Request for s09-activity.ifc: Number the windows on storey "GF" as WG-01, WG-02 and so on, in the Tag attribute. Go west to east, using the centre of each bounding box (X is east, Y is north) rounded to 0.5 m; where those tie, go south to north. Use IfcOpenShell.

First a look at what the model holds.

```python
import ifcopenshell
import ifcopenshell.util.element
import ifcopenshell.util.placement

model = ifcopenshell.open("s09-activity.ifc")
print(model.schema)
storey = next(s for s in model.by_type("IfcBuildingStorey") if s.Name == "GF")
windows = [e for e in ifcopenshell.util.element.get_decomposition(storey) if e.is_a("IfcWindow")]
for e in sorted(windows, key=lambda e: e.id()):
    origin = ifcopenshell.util.placement.get_local_placement(e.ObjectPlacement)[:3, 3]
    print(e.id(), e.Tag, e.Name, origin.round(2) + 0.0, sep=" | ")
```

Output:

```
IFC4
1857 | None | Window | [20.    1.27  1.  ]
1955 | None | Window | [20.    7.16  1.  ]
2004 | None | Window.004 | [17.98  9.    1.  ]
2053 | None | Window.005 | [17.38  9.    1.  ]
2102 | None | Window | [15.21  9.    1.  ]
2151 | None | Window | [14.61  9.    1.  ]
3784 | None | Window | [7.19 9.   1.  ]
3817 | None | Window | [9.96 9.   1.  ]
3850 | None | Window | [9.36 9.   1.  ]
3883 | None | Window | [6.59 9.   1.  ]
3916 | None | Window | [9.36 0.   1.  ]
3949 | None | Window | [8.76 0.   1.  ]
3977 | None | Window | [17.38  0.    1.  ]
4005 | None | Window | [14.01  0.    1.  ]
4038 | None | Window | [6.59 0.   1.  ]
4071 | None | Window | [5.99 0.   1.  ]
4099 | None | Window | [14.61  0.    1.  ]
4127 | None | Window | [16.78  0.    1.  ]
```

```python
import ifcopenshell
import ifcopenshell.geom
import ifcopenshell.util.element
import ifcopenshell.util.shape

model = ifcopenshell.open("s09-activity.ifc")
settings = ifcopenshell.geom.settings()
settings.set("use-world-coords", True)


def centre(element):
    shape = ifcopenshell.geom.create_shape(settings, element)
    return ifcopenshell.util.shape.get_bbox_centroid(shape.geometry)


storey = next(s for s in model.by_type("IfcBuildingStorey") if s.Name == "GF")
windows = [e for e in ifcopenshell.util.element.get_decomposition(storey) if e.is_a("IfcWindow")]

# Insertion points can sit at a corner or the storey origin, so sort by the geometry (in metres).
centres = {e: centre(e) for e in windows}
windows.sort(key=lambda e: (round(centres[e][0] / 0.5), centres[e][1]))

for i, e in enumerate(windows, start=1):
    number = f"WG-{i:02d}"
    e.Tag = number
    print(e.id(), number)

model.write("s09-activity_edited.ifc")
```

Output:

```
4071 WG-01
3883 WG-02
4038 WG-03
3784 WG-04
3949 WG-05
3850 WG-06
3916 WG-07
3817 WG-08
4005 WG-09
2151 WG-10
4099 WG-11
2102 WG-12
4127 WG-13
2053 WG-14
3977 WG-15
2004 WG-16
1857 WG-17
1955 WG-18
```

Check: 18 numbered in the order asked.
